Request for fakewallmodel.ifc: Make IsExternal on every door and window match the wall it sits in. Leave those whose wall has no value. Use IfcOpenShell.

First a look at what the model holds.

```python
import ifcopenshell
import ifcopenshell.util.element

model = ifcopenshell.open("fakewallmodel.ifc")
print(model.schema)
seen = {}
for e in model.by_type("IfcDoor") + model.by_type("IfcWindow"):
    if not e.FillsVoids:
        continue
    host = e.FillsVoids[0].RelatingOpeningElement.VoidsElements[0].RelatingBuildingElement
    own = ifcopenshell.util.element.get_pset(e, f"Pset_{e.is_a()[3:].removesuffix('StandardCase')}Common", "IsExternal")
    wall = ifcopenshell.util.element.get_pset(host, "Pset_WallCommon", "IsExternal")
    seen[e.is_a(), own, wall] = seen.get((e.is_a(), own, wall), 0) + 1
for (cls, own, wall), count in sorted(seen.items(), key=str):
    print(count, cls, "IsExternal:", own, "| host wall:", wall)
```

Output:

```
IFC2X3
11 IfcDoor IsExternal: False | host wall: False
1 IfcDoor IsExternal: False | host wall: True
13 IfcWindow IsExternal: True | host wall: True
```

```python
import ifcopenshell
import ifcopenshell.api.pset
import ifcopenshell.util.element

model = ifcopenshell.open("fakewallmodel.ifc")

count = 0
for ifc_class, pset_name in (("IfcDoor", "Pset_DoorCommon"), ("IfcWindow", "Pset_WindowCommon")):
    for e in model.by_type(ifc_class):
        if not e.FillsVoids:
            continue
        host = e.FillsVoids[0].RelatingOpeningElement.VoidsElements[0].RelatingBuildingElement
        external = ifcopenshell.util.element.get_pset(host, "Pset_WallCommon", "IsExternal")
        if external is None or ifcopenshell.util.element.get_pset(e, pset_name, "IsExternal") == external:
            continue
        pset = ifcopenshell.api.pset.add_pset(model, product=e, name=pset_name)
        ifcopenshell.api.pset.edit_pset(model, pset=pset, properties={"IsExternal": external})
        count += 1

print(count, "updated")

model.write("fakewallmodel_v2.ifc")
```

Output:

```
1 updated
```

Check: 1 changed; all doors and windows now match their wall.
